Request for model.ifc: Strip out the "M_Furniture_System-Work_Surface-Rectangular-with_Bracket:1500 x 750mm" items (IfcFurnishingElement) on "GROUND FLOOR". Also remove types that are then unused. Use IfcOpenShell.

First a look at what the model holds.

```python
import ifcopenshell
import ifcopenshell.util.element

model = ifcopenshell.open("model.ifc")
print(model.schema)
storey = next(s for s in model.by_type("IfcBuildingStorey") if s.Name == "GROUND FLOOR")
furniture = [e for e in ifcopenshell.util.element.get_decomposition(storey) if e.is_a("IfcFurnishingElement")]
seen = {}
for e in furniture:
    element_type = ifcopenshell.util.element.get_type(e)
    name = element_type.Name if element_type not in (None, e) else None
    seen[name] = seen.get(name, 0) + 1
for name, count in sorted(seen.items(), key=str):
    print(count, "x", name)
```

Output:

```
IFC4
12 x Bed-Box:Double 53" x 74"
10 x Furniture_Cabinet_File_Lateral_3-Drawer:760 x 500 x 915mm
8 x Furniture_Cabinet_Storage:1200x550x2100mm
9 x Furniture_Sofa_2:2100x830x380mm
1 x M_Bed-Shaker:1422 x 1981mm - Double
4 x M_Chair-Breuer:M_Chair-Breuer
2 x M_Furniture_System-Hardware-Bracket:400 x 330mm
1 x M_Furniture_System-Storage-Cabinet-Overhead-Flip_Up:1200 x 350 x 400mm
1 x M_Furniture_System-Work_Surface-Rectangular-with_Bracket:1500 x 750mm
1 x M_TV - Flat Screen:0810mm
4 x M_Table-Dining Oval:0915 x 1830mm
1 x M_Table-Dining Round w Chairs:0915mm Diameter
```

```python
import ifcopenshell
import ifcopenshell.api.root
import ifcopenshell.util.element

model = ifcopenshell.open("model.ifc")

storey = next(s for s in model.by_type("IfcBuildingStorey") if s.Name == "GROUND FLOOR")
furniture = [e for e in ifcopenshell.util.element.get_decomposition(storey) if e.is_a("IfcFurnishingElement")]
targets = [e for e in furniture if (t := ifcopenshell.util.element.get_type(e)) not in (None, e) and t.Name == "M_Furniture_System-Work_Surface-Rectangular-with_Bracket:1500 x 750mm"]
types = {ifcopenshell.util.element.get_type(e) for e in targets} - {None, *targets}

for e in targets:
    ifcopenshell.api.root.remove_product(model, product=e)
print(len(targets), "removed")

unused = [t for t in types if not ifcopenshell.util.element.get_types(t)]
for t in unused:
    ifcopenshell.api.root.remove_product(model, product=t)
print(len(unused), "unused types removed")

model.write("model_updated.ifc")
```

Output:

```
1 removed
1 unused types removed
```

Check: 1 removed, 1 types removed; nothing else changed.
